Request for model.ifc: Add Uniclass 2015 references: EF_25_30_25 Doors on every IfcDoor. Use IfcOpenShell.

First a look at what the model holds.

```python
import ifcopenshell

model = ifcopenshell.open("model.ifc")
print(model.schema)
print("classifications:", [c.Name for c in model.by_type("IfcClassification")])
for ifc_class in ("IfcDoor", "IfcRoof", "IfcStair", "IfcWall", "IfcWindow"):
    print(ifc_class, len(model.by_type(ifc_class)))
```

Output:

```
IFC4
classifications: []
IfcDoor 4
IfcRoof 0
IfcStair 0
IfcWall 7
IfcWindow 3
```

```python
import ifcopenshell
import ifcopenshell.api.classification

model = ifcopenshell.open("model.ifc")

system = ifcopenshell.api.classification.add_classification(model, classification="Uniclass 2015")

codes = {
    "IfcDoor": ("EF_25_30_25", "Doors"),
}
for ifc_class, (code, name) in codes.items():
    products = model.by_type(ifc_class)
    ifcopenshell.api.classification.add_reference(
        model, products=products, classification=system, identification=code, name=name
    )
    print(code, len(products))

model.write("model_updated.ifc")
```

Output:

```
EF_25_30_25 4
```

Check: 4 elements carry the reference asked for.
